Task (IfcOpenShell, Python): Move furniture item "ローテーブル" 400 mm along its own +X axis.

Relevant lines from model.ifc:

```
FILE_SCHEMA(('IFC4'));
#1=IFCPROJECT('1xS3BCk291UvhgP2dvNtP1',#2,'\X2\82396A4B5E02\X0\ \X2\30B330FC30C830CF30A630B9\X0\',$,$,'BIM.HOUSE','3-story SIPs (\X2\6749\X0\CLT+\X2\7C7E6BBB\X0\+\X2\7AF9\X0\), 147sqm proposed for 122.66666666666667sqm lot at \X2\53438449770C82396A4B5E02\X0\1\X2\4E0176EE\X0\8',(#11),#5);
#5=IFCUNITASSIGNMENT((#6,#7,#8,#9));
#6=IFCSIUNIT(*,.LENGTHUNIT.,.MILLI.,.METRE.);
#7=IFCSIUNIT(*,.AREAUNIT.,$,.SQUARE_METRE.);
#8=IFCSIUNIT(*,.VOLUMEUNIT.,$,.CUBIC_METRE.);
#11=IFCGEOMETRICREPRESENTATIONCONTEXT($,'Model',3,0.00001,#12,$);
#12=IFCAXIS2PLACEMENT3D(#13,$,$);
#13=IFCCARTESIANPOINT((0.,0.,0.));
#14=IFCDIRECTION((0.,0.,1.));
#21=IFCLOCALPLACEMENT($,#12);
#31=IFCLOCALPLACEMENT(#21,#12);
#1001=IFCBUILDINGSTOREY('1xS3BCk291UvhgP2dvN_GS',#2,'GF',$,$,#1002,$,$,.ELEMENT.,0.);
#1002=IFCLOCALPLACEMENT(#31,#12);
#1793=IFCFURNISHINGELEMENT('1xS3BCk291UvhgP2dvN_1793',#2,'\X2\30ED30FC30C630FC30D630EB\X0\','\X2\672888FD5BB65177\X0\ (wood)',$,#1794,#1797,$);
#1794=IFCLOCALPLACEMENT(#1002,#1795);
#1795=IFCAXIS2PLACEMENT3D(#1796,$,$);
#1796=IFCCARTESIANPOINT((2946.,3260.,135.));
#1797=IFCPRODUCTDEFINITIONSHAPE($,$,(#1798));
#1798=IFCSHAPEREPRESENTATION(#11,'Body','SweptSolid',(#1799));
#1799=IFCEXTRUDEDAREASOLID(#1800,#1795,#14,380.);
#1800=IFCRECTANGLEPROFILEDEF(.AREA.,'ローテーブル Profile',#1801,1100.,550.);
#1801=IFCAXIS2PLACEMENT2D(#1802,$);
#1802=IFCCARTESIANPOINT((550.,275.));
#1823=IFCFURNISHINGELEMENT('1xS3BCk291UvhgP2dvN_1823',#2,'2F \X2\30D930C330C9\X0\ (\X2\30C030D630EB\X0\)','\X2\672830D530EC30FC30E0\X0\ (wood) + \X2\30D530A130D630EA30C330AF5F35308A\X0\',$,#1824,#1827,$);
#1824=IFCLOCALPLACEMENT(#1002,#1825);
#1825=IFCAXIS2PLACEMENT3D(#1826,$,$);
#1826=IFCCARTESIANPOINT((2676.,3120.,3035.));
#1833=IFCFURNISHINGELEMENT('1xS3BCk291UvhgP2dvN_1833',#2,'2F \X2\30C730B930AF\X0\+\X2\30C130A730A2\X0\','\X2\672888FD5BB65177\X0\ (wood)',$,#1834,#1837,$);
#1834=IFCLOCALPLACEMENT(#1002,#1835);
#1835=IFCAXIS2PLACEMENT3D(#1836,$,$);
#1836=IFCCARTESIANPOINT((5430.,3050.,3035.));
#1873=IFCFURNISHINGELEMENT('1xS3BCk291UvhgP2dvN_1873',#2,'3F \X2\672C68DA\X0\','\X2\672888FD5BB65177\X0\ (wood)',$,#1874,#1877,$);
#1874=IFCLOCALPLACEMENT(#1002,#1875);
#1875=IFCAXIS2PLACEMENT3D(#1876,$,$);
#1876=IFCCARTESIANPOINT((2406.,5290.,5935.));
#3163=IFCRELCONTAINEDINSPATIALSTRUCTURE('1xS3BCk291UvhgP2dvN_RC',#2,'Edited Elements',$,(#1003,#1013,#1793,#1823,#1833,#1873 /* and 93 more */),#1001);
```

```python
import ifcopenshell
import ifcopenshell.api.geometry
import ifcopenshell.util.placement
import ifcopenshell.util.unit

model = ifcopenshell.open("model.ifc")
unit_scale = ifcopenshell.util.unit.calculate_unit_scale(model)

item = model.by_guid("1xS3BCk291UvhgP2dvN_1793")
matrix = ifcopenshell.util.placement.get_local_placement(item.ObjectPlacement)
matrix[:3, 3] += matrix[:3, 0] * 0.4 / unit_scale
ifcopenshell.api.geometry.edit_object_placement(model, product=item, matrix=matrix, is_si=False)

print(ifcopenshell.util.placement.get_local_placement(item.ObjectPlacement).round(3) + 0.0)

model.write("model_edited.ifc")
```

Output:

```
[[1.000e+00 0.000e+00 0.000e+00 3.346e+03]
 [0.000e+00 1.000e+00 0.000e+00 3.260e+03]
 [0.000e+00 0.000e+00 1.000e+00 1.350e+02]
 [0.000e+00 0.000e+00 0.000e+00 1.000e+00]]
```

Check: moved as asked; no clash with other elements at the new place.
